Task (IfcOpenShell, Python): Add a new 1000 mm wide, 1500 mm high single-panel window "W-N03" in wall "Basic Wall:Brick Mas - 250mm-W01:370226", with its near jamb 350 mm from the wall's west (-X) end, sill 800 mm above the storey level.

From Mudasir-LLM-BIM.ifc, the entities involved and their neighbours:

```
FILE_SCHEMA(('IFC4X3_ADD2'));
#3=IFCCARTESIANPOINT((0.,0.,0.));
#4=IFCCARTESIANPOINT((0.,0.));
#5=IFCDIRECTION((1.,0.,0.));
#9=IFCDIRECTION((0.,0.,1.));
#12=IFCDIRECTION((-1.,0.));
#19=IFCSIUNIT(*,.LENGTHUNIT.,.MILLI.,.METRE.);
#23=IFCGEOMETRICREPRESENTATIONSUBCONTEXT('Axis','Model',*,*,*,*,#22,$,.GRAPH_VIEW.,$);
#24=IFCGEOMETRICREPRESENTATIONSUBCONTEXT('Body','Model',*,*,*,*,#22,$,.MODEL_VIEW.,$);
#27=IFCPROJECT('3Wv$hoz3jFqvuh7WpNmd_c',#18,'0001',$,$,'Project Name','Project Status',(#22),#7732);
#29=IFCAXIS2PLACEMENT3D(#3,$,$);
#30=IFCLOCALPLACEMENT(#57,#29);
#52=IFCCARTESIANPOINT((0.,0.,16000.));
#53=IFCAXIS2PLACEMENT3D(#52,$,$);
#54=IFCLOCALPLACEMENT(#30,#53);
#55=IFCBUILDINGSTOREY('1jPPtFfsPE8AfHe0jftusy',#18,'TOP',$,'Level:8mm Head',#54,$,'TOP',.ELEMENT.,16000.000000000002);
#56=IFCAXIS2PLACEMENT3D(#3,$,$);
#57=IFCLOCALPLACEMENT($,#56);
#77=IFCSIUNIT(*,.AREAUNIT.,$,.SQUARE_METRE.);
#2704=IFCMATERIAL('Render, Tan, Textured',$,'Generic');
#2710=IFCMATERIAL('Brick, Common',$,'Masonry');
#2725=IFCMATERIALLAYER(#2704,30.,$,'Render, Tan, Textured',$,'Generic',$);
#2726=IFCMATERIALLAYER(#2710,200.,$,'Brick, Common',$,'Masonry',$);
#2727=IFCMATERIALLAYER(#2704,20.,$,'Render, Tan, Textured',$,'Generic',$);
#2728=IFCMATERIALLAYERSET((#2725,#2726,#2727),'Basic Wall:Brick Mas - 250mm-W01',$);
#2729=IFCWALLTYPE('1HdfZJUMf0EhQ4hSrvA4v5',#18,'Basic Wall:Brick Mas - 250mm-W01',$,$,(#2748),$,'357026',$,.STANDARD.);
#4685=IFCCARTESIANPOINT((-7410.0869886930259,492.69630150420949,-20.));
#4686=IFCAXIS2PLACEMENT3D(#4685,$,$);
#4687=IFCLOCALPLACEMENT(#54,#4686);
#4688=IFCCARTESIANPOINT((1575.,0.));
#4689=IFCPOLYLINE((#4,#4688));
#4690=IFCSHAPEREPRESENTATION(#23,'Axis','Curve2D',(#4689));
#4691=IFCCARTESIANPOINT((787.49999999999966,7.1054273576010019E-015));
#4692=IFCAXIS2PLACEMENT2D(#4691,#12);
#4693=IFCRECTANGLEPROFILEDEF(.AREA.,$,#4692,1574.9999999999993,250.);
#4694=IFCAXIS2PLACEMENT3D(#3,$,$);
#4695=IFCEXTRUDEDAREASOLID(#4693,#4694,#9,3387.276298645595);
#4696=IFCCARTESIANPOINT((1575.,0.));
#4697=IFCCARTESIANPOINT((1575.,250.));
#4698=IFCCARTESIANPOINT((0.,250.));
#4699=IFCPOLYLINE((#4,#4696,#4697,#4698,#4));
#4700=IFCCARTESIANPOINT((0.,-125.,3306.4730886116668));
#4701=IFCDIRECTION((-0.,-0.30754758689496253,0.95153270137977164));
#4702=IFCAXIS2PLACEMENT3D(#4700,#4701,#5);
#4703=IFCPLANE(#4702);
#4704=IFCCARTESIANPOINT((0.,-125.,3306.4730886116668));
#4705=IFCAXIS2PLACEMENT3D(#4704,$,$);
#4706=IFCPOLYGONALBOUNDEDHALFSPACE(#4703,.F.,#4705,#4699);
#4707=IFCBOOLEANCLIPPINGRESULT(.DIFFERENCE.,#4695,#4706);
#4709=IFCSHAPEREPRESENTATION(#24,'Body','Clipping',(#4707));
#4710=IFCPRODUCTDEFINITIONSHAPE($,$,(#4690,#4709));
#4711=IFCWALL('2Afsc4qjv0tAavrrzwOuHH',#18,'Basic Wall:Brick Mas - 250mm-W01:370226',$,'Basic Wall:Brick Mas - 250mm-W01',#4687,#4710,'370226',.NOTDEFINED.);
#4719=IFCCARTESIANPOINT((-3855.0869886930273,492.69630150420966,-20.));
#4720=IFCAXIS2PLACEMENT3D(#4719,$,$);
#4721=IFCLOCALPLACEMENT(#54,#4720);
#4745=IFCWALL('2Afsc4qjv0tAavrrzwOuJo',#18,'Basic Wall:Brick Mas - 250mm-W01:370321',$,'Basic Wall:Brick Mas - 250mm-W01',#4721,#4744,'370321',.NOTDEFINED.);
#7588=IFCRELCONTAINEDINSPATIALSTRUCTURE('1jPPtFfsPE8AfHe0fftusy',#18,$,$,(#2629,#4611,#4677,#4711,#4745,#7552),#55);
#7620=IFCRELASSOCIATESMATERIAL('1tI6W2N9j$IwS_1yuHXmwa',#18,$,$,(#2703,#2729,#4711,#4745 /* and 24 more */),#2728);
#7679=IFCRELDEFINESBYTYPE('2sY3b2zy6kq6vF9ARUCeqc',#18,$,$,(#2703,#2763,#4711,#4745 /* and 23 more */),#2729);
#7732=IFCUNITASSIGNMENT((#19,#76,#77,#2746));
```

```python
import numpy as np
import ifcopenshell
import ifcopenshell.api.feature
import ifcopenshell.api.geometry
import ifcopenshell.api.root
import ifcopenshell.api.spatial
import ifcopenshell.geom
import ifcopenshell.util.element
import ifcopenshell.util.placement
import ifcopenshell.util.representation
import ifcopenshell.util.shape
import ifcopenshell.util.unit

model = ifcopenshell.open("Mudasir-LLM-BIM.ifc")
unit_scale = ifcopenshell.util.unit.calculate_unit_scale(model)
settings = ifcopenshell.geom.settings()


def volume(element):
    """Net volume in cubic metres, openings subtracted."""
    shape = ifcopenshell.geom.create_shape(settings, element)
    return ifcopenshell.util.shape.get_volume(shape.geometry)


wall = model.by_id(4711)
storey = ifcopenshell.util.element.get_container(wall, ifc_class="IfcBuildingStorey")
context = ifcopenshell.util.representation.get_context(model, "Model", "Body", "MODEL_VIEW")
before = volume(wall)

width, height, from_end, sill = 1, 1.5, 0.35, 0.8  # metres

# The wall runs along its own X axis, and the end named is its -X end.
wall_shape = ifcopenshell.geom.create_shape(settings, wall)
x, y, z = ifcopenshell.util.shape.get_vertices(wall_shape.geometry).T
start = x.min() + from_end
face, thickness = float(y.min()), float(y.max() - y.min())
wall_matrix = ifcopenshell.util.placement.get_local_placement(wall.ObjectPlacement)
level = ifcopenshell.util.placement.get_local_placement(storey.ObjectPlacement)[2, 3]


def in_wall(x, y):
    """Placement at x, y metres in the wall's axes, at sill height."""
    matrix = wall_matrix.copy()
    matrix[:, 3] = wall_matrix @ np.array([x / unit_scale, y / unit_scale, 0.0, 1.0])
    matrix[2, 3] = level + sill / unit_scale
    return matrix


# Opening: a box that overshoots both wall faces by 50 mm.
opening = ifcopenshell.api.root.create_entity(model, ifc_class="IfcOpeningElement", predefined_type="OPENING")
box = ifcopenshell.api.geometry.add_wall_representation(
    model, context=context, length=width, height=height, thickness=thickness + 0.1
)
ifcopenshell.api.geometry.assign_representation(model, product=opening, representation=box)
ifcopenshell.api.geometry.edit_object_placement(model, product=opening, matrix=in_wall(start, face - 0.05), is_si=False)
ifcopenshell.api.feature.add_feature(model, feature=opening, element=wall)

window = ifcopenshell.api.root.create_entity(model, ifc_class="IfcWindow", name="W-N03", predefined_type="WINDOW")
window.OverallWidth, window.OverallHeight = width / unit_scale, height / unit_scale
window.PartitioningType = "SINGLE_PANEL"
body = ifcopenshell.api.geometry.add_window_representation(
    model,
    context=context,
    overall_width=window.OverallWidth,
    overall_height=window.OverallHeight,
    partition_type="SINGLE_PANEL",
)
ifcopenshell.api.geometry.assign_representation(model, product=window, representation=body)
ifcopenshell.api.spatial.assign_container(model, products=[window], relating_structure=storey)
ifcopenshell.api.feature.add_filling(model, opening=opening, element=window)

# Centre the window in the wall's thickness.
ifcopenshell.api.geometry.edit_object_placement(model, product=window, matrix=in_wall(start, face), is_si=False)
window_shape = ifcopenshell.geom.create_shape(settings, window)
depth = ifcopenshell.util.shape.get_vertices(window_shape.geometry)[:, 1]
offset = face + thickness / 2 - (depth.min() + depth.max()) / 2
ifcopenshell.api.geometry.edit_object_placement(model, product=window, matrix=in_wall(start, offset), is_si=False)

after = volume(wall)

print(f"wall volume {before:.3f} -> {after:.3f} m3")

model.write("Mudasir-LLM-BIM_v2.ifc")
```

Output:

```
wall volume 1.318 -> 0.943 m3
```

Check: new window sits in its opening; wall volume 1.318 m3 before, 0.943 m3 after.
